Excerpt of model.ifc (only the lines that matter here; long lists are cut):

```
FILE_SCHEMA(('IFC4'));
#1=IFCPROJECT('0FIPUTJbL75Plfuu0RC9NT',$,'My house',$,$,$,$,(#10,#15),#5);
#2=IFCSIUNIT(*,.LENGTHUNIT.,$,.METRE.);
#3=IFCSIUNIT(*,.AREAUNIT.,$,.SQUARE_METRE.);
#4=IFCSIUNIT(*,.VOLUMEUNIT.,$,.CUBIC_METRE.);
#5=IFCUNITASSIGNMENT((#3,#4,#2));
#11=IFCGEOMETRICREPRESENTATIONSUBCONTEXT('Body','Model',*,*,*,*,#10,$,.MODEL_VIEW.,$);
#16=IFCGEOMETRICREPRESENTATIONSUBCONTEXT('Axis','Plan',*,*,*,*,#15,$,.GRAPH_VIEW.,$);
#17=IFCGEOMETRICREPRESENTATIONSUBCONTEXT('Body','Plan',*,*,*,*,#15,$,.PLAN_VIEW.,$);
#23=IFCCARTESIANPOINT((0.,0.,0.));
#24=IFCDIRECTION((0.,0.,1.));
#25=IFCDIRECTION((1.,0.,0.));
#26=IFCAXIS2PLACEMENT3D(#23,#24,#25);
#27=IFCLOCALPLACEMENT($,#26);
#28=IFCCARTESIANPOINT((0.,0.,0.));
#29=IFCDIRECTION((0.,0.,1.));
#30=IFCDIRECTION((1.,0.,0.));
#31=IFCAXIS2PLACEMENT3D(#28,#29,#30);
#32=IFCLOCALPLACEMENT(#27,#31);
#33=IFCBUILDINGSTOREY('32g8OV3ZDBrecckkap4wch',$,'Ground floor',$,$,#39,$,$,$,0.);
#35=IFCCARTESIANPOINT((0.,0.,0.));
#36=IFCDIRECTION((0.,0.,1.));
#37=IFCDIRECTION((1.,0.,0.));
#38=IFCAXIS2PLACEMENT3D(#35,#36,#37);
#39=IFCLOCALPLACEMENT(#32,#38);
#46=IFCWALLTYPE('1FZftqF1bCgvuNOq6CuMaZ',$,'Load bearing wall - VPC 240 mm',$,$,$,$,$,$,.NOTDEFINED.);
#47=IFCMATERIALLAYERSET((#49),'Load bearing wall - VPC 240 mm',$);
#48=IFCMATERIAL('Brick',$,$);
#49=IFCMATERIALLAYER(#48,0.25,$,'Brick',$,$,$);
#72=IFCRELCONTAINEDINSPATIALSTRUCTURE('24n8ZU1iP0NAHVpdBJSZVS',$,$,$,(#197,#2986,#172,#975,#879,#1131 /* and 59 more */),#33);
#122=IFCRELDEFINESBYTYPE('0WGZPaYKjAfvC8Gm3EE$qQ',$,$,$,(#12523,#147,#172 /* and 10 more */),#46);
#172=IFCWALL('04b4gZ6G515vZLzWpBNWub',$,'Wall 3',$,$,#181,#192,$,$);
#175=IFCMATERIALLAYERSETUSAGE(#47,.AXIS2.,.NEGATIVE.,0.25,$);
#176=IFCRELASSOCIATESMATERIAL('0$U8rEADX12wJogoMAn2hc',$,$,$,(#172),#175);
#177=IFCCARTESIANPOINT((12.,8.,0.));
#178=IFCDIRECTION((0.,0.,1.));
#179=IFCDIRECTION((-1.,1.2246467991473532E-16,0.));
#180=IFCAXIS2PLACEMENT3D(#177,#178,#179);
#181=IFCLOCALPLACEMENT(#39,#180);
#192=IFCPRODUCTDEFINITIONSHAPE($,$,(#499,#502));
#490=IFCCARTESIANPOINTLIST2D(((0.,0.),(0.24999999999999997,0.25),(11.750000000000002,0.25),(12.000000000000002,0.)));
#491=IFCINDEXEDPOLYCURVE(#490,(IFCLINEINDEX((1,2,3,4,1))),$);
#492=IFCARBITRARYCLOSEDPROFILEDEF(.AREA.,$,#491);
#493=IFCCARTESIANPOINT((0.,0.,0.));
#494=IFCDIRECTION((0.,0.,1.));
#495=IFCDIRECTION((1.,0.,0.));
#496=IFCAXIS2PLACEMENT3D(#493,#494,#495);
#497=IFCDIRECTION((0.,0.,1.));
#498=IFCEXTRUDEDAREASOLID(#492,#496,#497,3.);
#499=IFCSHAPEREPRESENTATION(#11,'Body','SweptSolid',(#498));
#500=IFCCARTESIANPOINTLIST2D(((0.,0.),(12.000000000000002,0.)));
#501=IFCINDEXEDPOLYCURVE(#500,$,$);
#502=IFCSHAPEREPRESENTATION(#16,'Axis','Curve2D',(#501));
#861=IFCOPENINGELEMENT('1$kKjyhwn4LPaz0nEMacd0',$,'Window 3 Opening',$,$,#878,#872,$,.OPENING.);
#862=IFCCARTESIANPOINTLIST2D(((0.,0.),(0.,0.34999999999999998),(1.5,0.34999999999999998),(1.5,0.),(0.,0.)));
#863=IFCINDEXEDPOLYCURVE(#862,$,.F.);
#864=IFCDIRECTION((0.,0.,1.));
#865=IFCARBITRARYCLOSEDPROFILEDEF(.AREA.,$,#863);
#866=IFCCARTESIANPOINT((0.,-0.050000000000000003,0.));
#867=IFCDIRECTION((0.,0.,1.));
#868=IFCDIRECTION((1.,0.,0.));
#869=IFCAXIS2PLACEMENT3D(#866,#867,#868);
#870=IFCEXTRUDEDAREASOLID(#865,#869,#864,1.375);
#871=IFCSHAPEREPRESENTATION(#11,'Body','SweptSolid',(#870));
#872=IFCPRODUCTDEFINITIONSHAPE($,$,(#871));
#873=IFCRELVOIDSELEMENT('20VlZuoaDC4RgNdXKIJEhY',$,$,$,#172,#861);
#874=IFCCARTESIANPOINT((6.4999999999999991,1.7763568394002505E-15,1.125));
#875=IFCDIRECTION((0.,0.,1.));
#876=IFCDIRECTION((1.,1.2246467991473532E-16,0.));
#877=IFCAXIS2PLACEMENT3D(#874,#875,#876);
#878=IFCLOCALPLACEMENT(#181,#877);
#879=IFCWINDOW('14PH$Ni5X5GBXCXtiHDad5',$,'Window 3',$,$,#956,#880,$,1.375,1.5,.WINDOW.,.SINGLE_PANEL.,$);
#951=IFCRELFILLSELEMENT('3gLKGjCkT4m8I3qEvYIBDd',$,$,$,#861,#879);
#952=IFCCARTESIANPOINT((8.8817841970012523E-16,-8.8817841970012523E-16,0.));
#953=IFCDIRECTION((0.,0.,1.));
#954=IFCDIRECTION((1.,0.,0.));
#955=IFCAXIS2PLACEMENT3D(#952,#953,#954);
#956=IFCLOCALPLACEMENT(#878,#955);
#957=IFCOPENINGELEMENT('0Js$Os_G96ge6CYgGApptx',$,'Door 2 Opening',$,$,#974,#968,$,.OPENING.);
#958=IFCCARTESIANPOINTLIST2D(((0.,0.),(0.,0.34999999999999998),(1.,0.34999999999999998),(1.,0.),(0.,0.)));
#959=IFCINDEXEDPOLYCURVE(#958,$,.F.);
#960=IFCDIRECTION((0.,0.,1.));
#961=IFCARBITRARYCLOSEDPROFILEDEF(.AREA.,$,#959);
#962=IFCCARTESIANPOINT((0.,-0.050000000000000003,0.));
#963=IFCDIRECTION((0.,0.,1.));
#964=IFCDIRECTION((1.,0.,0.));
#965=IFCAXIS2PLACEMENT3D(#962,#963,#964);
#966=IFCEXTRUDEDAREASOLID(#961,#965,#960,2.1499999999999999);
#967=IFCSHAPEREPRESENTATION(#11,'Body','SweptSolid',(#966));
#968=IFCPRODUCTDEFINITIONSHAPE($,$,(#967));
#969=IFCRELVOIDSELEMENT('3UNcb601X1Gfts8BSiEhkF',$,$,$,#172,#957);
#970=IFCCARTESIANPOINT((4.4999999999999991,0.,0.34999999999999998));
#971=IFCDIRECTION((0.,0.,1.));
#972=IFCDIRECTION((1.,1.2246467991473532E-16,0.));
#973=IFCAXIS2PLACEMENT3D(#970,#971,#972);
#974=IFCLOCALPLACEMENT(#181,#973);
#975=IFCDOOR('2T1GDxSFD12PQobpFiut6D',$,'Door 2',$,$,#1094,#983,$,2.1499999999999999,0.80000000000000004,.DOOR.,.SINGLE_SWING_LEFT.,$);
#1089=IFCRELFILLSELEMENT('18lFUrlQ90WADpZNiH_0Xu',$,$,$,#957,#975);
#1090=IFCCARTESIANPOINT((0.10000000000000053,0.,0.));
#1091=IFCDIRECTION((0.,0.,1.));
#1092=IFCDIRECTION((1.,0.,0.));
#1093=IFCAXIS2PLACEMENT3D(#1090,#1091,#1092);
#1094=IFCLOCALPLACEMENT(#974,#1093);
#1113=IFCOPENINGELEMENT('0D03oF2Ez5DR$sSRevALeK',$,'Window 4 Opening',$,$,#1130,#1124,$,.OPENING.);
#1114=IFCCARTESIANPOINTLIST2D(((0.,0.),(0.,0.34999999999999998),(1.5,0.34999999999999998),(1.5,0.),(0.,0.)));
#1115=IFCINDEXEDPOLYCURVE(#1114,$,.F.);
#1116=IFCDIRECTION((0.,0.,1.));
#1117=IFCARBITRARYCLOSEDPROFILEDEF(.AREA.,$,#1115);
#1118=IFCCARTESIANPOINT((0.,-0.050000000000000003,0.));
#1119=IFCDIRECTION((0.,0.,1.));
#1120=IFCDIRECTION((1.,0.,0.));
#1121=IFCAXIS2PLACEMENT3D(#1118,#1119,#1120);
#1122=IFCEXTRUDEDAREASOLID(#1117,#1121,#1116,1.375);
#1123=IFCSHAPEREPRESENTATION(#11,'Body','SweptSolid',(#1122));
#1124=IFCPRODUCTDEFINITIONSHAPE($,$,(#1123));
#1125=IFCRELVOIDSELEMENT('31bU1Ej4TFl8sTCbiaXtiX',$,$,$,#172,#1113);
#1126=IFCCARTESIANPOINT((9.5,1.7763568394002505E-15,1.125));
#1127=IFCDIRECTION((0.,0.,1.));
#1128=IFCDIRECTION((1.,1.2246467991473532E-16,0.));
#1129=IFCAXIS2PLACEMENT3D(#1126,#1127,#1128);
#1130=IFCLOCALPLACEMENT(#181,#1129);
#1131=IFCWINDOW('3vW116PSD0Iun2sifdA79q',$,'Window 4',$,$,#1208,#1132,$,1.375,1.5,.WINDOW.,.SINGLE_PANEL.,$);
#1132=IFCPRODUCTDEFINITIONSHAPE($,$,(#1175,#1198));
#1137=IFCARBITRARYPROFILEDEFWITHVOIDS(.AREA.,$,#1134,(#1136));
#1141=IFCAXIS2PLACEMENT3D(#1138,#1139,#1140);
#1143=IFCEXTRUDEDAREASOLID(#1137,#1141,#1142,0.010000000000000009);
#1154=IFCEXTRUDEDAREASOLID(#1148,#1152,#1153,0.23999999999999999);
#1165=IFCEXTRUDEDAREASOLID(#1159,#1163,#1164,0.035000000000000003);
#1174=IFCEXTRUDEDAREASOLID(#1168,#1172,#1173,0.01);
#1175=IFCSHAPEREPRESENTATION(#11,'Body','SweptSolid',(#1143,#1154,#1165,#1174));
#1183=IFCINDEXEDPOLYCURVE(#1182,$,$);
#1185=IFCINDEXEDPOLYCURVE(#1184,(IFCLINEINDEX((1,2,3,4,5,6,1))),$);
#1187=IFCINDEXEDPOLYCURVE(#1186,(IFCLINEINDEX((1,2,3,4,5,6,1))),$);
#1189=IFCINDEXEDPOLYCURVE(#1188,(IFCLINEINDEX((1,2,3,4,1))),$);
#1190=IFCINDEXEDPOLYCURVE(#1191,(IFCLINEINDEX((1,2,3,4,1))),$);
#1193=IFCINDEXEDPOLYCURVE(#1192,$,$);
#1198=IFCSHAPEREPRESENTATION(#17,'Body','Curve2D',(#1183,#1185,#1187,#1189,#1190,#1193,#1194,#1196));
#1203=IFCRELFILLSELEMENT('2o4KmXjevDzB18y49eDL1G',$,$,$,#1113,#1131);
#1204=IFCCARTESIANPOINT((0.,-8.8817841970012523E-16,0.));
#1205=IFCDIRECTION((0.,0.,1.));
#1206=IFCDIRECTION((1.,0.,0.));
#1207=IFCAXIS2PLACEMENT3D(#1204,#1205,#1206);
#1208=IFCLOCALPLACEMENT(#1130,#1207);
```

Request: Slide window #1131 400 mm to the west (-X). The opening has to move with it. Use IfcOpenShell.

```python
import ifcopenshell
import ifcopenshell.api.geometry
import ifcopenshell.util.placement

model = ifcopenshell.open("model.ifc")

window = model.by_guid("3vW116PSD0Iun2sifdA79q")
opening = window.FillsVoids[0].RelatingOpeningElement
wall = opening.VoidsElements[0].RelatingBuildingElement

wall_matrix = ifcopenshell.util.placement.get_local_placement(wall.ObjectPlacement)
shift = wall_matrix[:3, 0] * 0.4
before = ifcopenshell.util.placement.get_local_placement(window.ObjectPlacement)[:3, 3].copy()

# The window is placed relative to its opening, so it follows when the opening moves.
matrix = ifcopenshell.util.placement.get_local_placement(opening.ObjectPlacement)
matrix[:3, 3] += shift
ifcopenshell.api.geometry.edit_object_placement(
    model, product=opening, matrix=matrix, is_si=False, should_transform_children=True
)

after = ifcopenshell.util.placement.get_local_placement(window.ObjectPlacement)[:3, 3]
print("window moved by", (after - before).round(3) + 0.0)

model.write("model_updated.ifc")
```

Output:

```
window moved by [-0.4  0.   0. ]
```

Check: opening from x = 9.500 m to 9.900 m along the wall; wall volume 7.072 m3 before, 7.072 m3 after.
